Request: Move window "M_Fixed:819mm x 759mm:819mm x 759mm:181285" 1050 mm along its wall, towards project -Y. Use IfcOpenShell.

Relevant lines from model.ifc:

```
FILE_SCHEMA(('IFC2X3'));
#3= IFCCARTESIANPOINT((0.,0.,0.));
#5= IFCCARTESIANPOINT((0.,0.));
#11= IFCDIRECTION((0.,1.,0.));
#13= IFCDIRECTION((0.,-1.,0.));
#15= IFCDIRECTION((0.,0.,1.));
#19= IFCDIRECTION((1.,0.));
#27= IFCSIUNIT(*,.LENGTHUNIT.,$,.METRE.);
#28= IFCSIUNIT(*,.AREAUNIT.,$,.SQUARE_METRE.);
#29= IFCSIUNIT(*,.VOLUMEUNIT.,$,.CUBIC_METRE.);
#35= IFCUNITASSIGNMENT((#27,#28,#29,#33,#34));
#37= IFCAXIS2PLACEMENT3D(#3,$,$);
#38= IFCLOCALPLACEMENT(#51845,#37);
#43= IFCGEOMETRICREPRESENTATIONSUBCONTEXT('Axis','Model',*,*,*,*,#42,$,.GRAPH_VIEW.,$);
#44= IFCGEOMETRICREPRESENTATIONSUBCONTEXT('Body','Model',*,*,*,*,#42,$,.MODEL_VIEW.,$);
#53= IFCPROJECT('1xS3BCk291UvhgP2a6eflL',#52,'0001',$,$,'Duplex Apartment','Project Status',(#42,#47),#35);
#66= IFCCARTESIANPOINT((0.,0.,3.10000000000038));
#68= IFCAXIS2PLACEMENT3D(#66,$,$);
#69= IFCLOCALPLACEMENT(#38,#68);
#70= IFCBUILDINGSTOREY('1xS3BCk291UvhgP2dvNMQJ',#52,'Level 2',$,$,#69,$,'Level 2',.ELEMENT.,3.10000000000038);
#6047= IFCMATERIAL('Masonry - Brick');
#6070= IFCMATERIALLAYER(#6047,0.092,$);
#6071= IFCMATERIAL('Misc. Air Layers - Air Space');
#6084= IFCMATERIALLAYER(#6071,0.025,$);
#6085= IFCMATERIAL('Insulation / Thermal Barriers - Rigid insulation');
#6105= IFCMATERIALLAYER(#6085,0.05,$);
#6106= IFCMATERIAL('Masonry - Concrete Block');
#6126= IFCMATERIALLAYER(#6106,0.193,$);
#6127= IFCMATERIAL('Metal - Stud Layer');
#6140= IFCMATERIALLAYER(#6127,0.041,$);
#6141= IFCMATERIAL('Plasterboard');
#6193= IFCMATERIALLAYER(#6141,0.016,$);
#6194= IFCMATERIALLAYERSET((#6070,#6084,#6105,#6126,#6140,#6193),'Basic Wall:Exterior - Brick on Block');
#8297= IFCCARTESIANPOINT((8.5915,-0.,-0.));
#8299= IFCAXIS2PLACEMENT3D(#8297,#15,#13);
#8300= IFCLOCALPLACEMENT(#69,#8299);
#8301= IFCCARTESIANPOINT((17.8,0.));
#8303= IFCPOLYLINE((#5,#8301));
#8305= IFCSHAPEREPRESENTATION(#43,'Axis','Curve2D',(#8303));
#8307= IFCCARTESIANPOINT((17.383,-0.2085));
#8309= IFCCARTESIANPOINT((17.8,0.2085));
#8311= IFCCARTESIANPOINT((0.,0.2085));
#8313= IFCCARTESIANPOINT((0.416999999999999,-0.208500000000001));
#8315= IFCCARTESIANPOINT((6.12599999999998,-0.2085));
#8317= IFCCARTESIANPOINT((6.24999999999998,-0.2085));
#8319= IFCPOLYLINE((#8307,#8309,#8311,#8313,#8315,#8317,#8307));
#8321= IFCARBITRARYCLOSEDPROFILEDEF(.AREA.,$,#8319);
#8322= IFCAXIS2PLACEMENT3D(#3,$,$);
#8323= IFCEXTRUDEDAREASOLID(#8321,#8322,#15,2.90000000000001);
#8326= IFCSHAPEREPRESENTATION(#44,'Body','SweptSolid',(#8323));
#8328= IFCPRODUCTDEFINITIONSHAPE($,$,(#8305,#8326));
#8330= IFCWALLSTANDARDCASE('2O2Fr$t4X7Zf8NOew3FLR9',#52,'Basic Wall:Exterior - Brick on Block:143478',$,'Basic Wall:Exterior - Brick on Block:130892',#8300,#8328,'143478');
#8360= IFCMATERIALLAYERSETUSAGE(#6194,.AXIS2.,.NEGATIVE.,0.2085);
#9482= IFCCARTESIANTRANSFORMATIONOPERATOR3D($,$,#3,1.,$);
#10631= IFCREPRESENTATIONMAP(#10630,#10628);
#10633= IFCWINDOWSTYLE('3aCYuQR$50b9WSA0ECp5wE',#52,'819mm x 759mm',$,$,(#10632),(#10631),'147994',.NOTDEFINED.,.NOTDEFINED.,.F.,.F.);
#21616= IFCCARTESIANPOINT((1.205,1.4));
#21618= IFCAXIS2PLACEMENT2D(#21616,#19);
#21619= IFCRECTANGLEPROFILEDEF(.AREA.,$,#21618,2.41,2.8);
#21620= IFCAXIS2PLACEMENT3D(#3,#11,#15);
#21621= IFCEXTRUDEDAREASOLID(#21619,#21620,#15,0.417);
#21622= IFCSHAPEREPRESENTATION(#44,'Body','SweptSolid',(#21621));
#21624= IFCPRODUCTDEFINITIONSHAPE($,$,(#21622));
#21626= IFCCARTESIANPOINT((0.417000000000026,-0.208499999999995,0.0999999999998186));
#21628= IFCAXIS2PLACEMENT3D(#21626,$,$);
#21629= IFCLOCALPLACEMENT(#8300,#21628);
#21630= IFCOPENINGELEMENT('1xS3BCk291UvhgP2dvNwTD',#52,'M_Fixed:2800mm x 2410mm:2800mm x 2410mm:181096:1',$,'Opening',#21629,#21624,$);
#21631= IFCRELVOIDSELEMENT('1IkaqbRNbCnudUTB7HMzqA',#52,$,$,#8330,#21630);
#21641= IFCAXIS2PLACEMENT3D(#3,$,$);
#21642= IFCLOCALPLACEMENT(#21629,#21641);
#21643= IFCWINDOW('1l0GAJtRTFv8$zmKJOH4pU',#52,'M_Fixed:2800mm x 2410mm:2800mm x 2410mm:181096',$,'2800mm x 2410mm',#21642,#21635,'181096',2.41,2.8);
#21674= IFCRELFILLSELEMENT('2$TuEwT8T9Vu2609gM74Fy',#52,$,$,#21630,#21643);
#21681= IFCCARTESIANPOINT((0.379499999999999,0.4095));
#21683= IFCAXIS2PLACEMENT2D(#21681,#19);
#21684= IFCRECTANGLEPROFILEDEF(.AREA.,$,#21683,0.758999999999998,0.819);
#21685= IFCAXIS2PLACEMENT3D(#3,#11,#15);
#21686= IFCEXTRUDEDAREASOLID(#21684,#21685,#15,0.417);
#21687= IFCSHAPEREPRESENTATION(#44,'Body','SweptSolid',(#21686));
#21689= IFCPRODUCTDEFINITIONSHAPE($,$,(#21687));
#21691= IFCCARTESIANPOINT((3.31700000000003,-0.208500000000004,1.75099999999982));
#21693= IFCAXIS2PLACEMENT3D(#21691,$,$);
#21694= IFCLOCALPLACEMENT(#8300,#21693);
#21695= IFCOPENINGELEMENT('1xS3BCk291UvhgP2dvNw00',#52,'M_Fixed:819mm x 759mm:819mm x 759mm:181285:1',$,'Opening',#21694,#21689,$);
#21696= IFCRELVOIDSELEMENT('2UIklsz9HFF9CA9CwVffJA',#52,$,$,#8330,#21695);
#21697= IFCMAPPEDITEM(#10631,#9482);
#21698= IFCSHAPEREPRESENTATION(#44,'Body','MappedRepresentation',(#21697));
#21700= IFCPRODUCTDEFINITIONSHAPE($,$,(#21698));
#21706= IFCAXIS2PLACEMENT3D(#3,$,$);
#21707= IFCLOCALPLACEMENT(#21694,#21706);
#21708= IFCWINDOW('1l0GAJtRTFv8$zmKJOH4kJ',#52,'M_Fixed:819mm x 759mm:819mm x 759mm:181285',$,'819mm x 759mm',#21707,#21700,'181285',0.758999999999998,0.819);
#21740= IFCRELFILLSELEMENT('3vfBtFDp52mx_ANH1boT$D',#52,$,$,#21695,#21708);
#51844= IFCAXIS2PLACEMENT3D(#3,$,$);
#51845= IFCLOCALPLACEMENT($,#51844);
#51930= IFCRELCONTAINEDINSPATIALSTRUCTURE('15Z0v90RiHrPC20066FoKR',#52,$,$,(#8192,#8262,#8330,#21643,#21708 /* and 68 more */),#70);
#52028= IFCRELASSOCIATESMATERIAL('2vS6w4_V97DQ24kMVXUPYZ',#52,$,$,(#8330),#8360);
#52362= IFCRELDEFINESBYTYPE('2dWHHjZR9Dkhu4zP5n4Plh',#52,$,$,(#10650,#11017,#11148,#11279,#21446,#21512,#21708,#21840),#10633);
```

```python
import ifcopenshell
import ifcopenshell.api.geometry
import ifcopenshell.util.placement
import ifcopenshell.util.unit

model = ifcopenshell.open("model.ifc")
unit_scale = ifcopenshell.util.unit.calculate_unit_scale(model)

window = model.by_guid("1l0GAJtRTFv8$zmKJOH4kJ")
opening = window.FillsVoids[0].RelatingOpeningElement
wall = opening.VoidsElements[0].RelatingBuildingElement

wall_matrix = ifcopenshell.util.placement.get_local_placement(wall.ObjectPlacement)
shift = wall_matrix[:3, 0] * 1.05 / unit_scale
before = ifcopenshell.util.placement.get_local_placement(window.ObjectPlacement)[:3, 3].copy()

# The window is placed relative to its opening, so it follows when the opening moves.
matrix = ifcopenshell.util.placement.get_local_placement(opening.ObjectPlacement)
matrix[:3, 3] += shift
ifcopenshell.api.geometry.edit_object_placement(
    model, product=opening, matrix=matrix, is_si=False, should_transform_children=True
)

after = ifcopenshell.util.placement.get_local_placement(window.ObjectPlacement)[:3, 3]
print("window moved by", (after - before).round(3) + 0.0)

model.write("model_v2.ifc")
```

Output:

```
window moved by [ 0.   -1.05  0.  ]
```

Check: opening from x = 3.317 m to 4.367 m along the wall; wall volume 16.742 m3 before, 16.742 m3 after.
